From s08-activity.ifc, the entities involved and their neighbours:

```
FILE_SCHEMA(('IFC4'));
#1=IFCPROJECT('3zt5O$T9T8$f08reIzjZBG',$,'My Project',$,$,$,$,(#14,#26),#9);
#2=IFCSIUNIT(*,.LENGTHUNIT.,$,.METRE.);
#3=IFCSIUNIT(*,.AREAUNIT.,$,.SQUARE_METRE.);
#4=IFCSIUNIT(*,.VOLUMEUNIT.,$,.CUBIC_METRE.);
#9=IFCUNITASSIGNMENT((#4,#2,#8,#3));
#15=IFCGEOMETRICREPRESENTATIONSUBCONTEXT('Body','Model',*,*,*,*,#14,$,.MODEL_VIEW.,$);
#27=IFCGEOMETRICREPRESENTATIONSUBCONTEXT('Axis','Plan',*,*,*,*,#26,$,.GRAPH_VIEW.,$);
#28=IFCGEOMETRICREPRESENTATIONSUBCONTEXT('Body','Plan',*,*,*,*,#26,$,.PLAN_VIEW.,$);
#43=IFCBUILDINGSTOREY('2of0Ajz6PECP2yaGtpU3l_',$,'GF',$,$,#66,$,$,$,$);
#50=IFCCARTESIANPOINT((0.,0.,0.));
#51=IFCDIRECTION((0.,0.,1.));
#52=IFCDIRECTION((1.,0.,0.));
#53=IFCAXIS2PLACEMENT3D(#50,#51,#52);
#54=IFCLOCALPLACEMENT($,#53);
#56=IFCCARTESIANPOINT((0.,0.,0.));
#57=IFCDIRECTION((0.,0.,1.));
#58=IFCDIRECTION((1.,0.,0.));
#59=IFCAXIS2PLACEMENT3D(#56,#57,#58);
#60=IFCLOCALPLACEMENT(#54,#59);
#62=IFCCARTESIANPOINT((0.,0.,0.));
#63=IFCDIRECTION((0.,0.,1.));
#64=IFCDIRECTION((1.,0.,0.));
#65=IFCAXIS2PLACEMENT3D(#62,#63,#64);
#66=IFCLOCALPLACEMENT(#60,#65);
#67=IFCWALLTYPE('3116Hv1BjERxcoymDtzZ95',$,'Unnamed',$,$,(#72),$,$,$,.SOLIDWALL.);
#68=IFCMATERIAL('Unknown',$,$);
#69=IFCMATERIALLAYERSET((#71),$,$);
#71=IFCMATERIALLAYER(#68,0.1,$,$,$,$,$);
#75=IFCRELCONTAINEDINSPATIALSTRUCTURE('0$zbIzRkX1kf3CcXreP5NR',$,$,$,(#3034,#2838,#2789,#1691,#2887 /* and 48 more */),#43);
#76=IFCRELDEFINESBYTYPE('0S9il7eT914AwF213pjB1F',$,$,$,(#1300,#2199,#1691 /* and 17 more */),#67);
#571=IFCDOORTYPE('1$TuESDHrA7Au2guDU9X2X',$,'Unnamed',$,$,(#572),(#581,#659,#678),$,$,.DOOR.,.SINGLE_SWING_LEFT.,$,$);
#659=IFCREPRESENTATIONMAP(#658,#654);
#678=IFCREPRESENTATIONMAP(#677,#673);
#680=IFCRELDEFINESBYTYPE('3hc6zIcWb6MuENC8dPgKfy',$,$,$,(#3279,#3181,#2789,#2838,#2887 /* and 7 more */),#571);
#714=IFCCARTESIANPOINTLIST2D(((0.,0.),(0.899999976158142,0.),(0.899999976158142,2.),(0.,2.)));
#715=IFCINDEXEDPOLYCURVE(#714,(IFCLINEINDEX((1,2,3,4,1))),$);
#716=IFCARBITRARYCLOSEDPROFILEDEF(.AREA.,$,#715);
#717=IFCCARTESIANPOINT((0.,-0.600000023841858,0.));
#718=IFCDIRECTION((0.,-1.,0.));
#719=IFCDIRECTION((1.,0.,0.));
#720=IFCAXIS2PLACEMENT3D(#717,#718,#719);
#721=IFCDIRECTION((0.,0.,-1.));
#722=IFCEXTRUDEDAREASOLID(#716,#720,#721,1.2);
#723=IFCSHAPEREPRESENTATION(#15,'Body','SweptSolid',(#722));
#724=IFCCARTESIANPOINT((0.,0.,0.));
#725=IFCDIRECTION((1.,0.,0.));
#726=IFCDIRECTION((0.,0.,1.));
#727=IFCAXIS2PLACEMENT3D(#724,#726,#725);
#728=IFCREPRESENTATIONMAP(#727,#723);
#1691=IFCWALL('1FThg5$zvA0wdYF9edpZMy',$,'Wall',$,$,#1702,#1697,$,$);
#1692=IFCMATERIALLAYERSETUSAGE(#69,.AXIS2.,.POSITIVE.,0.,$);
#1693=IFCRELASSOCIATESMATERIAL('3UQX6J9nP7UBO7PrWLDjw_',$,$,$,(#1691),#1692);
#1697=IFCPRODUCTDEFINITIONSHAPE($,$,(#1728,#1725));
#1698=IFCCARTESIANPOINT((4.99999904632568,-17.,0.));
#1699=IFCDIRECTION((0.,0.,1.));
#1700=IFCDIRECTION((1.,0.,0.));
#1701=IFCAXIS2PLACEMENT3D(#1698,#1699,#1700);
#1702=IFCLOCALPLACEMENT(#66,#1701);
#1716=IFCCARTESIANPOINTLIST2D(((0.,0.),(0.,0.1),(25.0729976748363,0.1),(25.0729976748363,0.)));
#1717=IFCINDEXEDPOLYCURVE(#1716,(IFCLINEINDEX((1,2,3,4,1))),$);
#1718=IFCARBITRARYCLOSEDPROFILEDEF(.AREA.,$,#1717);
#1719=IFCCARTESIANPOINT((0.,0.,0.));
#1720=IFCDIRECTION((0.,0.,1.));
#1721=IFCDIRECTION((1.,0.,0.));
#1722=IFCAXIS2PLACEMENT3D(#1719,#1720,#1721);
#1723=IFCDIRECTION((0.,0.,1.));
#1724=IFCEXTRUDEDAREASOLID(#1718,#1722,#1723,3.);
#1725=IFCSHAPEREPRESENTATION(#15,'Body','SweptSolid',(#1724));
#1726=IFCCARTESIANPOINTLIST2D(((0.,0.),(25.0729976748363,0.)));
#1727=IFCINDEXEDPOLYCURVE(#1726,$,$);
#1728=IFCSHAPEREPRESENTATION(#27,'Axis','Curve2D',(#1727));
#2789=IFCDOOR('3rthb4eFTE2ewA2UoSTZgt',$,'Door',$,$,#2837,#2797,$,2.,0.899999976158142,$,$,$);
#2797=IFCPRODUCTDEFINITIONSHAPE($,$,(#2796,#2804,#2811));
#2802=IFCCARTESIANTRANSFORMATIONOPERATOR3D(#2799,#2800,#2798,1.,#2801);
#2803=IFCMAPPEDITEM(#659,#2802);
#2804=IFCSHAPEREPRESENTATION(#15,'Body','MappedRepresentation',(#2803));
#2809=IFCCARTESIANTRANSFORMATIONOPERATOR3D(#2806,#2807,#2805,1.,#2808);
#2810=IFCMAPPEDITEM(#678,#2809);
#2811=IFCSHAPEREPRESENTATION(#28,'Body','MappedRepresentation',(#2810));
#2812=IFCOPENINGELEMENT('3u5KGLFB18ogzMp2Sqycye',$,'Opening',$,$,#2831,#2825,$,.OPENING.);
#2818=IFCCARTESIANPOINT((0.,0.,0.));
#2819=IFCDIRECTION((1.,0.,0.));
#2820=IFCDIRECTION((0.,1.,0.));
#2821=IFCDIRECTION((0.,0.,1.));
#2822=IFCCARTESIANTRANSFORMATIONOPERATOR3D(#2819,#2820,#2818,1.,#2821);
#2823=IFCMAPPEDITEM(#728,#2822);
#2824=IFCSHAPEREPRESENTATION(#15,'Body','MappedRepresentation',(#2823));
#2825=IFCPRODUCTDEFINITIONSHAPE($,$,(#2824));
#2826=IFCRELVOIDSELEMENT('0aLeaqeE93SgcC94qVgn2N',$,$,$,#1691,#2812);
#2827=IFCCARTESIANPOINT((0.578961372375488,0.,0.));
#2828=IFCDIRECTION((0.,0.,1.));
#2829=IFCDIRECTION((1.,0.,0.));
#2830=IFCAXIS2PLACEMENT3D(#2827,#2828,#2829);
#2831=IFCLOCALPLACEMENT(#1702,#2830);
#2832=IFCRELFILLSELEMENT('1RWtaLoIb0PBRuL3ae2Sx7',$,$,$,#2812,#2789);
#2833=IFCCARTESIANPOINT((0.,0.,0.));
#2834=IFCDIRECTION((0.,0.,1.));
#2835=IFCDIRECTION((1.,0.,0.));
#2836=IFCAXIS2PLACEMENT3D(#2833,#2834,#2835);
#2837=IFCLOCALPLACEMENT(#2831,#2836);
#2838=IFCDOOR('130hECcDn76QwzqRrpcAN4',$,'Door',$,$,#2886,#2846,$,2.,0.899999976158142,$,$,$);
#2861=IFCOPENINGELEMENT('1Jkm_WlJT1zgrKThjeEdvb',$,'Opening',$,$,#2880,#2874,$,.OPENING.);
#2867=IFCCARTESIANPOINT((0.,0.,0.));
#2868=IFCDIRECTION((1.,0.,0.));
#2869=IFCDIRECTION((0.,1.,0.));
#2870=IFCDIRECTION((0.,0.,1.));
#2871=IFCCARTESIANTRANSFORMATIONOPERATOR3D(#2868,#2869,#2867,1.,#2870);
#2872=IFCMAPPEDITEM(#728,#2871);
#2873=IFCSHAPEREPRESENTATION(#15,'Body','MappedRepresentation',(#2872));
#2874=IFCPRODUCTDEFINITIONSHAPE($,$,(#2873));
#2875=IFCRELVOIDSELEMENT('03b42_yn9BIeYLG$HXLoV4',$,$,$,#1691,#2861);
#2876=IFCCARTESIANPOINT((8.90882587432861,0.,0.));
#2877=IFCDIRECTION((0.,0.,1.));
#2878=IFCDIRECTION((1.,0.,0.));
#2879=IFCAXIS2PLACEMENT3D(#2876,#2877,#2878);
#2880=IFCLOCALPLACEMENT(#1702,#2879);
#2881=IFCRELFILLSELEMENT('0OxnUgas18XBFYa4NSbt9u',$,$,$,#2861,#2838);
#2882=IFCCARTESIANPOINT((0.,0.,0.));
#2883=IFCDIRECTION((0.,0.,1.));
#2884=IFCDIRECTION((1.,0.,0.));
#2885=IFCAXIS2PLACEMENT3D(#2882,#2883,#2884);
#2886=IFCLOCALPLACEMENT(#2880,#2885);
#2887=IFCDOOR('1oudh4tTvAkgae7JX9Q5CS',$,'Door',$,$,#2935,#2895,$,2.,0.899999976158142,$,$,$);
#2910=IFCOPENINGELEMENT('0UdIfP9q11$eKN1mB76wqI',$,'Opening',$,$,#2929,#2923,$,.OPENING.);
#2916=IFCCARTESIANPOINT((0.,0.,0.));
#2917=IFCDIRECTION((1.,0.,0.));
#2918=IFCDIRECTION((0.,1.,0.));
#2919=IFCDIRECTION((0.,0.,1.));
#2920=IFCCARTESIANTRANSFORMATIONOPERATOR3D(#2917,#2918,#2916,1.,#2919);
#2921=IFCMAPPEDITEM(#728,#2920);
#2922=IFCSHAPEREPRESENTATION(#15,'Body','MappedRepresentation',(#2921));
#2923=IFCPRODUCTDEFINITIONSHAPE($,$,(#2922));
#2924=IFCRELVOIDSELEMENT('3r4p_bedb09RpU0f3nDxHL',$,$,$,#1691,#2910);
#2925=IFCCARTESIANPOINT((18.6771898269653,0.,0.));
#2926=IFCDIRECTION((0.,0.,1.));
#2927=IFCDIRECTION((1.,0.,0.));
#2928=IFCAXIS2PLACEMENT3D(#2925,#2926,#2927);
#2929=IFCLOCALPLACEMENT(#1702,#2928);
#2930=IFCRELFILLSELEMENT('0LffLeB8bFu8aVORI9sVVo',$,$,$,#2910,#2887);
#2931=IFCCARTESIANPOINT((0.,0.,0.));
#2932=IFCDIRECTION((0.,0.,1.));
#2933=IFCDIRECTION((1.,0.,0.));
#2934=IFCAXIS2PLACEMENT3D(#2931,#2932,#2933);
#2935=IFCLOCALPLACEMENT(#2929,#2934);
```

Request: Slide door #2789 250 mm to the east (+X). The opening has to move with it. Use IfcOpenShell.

```python
import ifcopenshell
import ifcopenshell.api.geometry
import ifcopenshell.util.placement
import ifcopenshell.util.unit

model = ifcopenshell.open("s08-activity.ifc")
unit_scale = ifcopenshell.util.unit.calculate_unit_scale(model)

door = model.by_id(2789)
opening = door.FillsVoids[0].RelatingOpeningElement
wall = opening.VoidsElements[0].RelatingBuildingElement

wall_matrix = ifcopenshell.util.placement.get_local_placement(wall.ObjectPlacement)
shift = wall_matrix[:3, 0] * 0.25 / unit_scale
before = ifcopenshell.util.placement.get_local_placement(door.ObjectPlacement)[:3, 3].copy()

# The door is placed relative to its opening, so it follows when the opening moves.
matrix = ifcopenshell.util.placement.get_local_placement(opening.ObjectPlacement)
matrix[:3, 3] += shift
ifcopenshell.api.geometry.edit_object_placement(
    model, product=opening, matrix=matrix, is_si=False, should_transform_children=True
)

after = ifcopenshell.util.placement.get_local_placement(door.ObjectPlacement)[:3, 3]
print("door moved by", (after - before).round(3) + 0.0)

model.write("s08-activity_v2.ifc")
```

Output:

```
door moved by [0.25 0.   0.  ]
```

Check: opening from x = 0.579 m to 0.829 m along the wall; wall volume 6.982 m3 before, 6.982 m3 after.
